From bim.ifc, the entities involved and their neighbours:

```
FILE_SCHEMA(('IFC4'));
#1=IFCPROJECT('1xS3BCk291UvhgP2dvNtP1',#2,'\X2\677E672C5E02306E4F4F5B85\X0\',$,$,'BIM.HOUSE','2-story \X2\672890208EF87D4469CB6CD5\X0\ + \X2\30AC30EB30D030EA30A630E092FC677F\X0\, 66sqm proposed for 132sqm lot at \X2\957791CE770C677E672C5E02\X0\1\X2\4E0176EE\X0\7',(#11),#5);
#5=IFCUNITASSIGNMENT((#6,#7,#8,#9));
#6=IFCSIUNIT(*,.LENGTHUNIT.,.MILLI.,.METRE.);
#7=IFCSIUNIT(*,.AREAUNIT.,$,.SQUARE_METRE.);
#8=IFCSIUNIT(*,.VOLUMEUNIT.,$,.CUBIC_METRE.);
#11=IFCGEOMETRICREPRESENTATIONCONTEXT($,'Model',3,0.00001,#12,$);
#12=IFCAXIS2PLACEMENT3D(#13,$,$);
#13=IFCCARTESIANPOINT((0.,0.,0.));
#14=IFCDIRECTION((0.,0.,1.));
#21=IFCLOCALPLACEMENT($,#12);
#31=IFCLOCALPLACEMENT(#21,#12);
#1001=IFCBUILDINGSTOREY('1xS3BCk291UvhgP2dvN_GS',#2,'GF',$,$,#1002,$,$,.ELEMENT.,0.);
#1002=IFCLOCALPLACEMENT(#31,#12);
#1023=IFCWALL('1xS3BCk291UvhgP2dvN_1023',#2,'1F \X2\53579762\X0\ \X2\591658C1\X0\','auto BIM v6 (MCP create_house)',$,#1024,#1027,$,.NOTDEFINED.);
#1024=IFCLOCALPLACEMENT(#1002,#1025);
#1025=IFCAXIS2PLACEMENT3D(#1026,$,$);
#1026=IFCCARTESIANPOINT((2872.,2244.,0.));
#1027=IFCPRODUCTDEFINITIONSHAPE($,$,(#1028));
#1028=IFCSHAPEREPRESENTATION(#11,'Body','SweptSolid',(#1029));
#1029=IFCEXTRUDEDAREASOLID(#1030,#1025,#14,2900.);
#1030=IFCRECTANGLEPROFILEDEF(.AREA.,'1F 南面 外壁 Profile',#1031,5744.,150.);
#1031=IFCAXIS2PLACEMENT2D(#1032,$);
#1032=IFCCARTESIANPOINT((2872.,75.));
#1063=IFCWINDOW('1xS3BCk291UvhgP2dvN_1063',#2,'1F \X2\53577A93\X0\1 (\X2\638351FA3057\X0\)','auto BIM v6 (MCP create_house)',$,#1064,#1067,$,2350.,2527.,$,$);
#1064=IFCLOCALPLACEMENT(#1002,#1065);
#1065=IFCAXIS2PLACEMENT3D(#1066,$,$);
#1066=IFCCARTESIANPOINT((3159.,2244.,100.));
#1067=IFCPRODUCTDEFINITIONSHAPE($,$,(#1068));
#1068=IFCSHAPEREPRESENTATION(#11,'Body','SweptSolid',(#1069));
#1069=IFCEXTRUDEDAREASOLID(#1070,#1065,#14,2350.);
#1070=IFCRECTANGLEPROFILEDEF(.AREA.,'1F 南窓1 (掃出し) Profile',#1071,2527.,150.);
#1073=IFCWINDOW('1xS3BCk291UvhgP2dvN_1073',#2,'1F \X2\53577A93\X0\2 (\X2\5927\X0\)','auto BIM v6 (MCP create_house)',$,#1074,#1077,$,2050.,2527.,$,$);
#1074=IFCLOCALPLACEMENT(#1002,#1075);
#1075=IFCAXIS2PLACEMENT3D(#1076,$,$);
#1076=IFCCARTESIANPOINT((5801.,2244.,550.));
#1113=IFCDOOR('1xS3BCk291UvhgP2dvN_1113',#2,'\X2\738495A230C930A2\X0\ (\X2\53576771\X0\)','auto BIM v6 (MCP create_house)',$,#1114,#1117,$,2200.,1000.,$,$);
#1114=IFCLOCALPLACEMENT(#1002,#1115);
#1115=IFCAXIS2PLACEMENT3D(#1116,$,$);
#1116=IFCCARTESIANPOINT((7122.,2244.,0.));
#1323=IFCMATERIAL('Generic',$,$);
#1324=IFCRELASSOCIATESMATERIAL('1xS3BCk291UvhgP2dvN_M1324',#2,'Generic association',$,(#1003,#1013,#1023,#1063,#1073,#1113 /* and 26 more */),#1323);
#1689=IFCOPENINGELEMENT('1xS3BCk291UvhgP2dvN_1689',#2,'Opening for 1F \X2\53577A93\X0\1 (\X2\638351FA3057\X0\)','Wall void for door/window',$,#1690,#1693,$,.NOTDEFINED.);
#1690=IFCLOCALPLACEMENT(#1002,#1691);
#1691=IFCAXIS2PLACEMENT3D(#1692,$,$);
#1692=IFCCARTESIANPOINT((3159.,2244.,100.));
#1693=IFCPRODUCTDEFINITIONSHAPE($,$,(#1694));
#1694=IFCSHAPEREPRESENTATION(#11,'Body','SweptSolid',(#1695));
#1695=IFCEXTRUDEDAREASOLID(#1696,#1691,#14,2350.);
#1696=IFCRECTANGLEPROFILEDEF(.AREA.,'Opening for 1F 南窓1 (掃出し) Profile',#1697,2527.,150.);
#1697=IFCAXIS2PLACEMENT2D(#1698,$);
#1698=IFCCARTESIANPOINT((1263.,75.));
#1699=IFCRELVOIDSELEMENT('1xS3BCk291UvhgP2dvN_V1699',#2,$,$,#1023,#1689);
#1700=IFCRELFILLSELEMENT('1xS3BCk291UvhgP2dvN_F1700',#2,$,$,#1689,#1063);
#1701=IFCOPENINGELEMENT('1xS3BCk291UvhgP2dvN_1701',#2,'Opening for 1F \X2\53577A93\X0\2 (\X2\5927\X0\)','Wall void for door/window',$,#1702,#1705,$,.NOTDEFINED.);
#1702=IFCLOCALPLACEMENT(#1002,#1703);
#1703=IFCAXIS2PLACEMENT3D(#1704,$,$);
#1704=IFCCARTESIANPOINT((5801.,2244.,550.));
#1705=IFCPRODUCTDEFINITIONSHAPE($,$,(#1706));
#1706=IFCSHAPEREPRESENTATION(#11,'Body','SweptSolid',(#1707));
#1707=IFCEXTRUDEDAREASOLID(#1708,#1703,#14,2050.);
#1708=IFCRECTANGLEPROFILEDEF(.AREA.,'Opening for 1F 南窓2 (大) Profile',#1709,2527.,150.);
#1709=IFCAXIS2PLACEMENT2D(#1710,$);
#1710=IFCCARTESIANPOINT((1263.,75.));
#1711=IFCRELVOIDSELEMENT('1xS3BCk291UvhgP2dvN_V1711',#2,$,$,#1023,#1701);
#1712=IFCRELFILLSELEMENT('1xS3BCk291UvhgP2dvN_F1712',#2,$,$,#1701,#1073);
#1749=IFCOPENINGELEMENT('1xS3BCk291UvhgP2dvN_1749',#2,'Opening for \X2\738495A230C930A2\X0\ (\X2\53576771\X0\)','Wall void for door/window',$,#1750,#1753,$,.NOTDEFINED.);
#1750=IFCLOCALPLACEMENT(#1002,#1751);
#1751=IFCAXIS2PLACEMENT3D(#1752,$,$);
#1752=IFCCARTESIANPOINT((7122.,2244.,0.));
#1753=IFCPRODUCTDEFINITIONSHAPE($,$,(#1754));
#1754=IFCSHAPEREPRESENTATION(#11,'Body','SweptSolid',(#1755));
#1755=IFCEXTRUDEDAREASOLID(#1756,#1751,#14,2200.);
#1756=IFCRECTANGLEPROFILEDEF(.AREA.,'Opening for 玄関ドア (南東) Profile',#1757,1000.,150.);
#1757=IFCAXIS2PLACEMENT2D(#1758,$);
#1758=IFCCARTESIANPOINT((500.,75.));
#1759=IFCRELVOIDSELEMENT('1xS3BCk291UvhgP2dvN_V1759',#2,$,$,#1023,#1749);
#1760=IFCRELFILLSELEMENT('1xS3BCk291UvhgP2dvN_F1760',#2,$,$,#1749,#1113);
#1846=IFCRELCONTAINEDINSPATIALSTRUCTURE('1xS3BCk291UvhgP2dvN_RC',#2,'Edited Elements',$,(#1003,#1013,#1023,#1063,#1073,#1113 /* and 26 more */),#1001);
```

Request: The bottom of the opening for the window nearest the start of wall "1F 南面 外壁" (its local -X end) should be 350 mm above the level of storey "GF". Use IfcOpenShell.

```python
import numpy as np
import ifcopenshell
import ifcopenshell.api.geometry
import ifcopenshell.geom
import ifcopenshell.util.element
import ifcopenshell.util.placement
import ifcopenshell.util.shape
import ifcopenshell.util.unit

model = ifcopenshell.open("bim.ifc")
unit_scale = ifcopenshell.util.unit.calculate_unit_scale(model)

window = model.by_id(1063)
opening = window.FillsVoids[0].RelatingOpeningElement
storey = ifcopenshell.util.element.get_container(window, ifc_class="IfcBuildingStorey")
level = ifcopenshell.util.placement.get_local_placement(storey.ObjectPlacement)[2, 3]

# The opening's origin need not be at the sill, so measure its lowest point.
shape = ifcopenshell.geom.create_shape(ifcopenshell.geom.settings(), opening)
bottom = ifcopenshell.util.shape.get_shape_bottom_elevation(shape, shape.geometry) / unit_scale
dz = level + 0.35 / unit_scale - bottom

shift = np.array([0.0, 0.0, dz])
# The window is not placed relative to its opening, so move both.
for product in (opening, window):
    matrix = ifcopenshell.util.placement.get_local_placement(product.ObjectPlacement)
    matrix[:3, 3] += shift
    ifcopenshell.api.geometry.edit_object_placement(model, product=product, matrix=matrix, is_si=False)

print(f"moved by {dz * unit_scale:+.3f} m")

model.write("bim_updated.ifc")
```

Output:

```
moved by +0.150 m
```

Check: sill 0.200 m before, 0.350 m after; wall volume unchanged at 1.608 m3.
